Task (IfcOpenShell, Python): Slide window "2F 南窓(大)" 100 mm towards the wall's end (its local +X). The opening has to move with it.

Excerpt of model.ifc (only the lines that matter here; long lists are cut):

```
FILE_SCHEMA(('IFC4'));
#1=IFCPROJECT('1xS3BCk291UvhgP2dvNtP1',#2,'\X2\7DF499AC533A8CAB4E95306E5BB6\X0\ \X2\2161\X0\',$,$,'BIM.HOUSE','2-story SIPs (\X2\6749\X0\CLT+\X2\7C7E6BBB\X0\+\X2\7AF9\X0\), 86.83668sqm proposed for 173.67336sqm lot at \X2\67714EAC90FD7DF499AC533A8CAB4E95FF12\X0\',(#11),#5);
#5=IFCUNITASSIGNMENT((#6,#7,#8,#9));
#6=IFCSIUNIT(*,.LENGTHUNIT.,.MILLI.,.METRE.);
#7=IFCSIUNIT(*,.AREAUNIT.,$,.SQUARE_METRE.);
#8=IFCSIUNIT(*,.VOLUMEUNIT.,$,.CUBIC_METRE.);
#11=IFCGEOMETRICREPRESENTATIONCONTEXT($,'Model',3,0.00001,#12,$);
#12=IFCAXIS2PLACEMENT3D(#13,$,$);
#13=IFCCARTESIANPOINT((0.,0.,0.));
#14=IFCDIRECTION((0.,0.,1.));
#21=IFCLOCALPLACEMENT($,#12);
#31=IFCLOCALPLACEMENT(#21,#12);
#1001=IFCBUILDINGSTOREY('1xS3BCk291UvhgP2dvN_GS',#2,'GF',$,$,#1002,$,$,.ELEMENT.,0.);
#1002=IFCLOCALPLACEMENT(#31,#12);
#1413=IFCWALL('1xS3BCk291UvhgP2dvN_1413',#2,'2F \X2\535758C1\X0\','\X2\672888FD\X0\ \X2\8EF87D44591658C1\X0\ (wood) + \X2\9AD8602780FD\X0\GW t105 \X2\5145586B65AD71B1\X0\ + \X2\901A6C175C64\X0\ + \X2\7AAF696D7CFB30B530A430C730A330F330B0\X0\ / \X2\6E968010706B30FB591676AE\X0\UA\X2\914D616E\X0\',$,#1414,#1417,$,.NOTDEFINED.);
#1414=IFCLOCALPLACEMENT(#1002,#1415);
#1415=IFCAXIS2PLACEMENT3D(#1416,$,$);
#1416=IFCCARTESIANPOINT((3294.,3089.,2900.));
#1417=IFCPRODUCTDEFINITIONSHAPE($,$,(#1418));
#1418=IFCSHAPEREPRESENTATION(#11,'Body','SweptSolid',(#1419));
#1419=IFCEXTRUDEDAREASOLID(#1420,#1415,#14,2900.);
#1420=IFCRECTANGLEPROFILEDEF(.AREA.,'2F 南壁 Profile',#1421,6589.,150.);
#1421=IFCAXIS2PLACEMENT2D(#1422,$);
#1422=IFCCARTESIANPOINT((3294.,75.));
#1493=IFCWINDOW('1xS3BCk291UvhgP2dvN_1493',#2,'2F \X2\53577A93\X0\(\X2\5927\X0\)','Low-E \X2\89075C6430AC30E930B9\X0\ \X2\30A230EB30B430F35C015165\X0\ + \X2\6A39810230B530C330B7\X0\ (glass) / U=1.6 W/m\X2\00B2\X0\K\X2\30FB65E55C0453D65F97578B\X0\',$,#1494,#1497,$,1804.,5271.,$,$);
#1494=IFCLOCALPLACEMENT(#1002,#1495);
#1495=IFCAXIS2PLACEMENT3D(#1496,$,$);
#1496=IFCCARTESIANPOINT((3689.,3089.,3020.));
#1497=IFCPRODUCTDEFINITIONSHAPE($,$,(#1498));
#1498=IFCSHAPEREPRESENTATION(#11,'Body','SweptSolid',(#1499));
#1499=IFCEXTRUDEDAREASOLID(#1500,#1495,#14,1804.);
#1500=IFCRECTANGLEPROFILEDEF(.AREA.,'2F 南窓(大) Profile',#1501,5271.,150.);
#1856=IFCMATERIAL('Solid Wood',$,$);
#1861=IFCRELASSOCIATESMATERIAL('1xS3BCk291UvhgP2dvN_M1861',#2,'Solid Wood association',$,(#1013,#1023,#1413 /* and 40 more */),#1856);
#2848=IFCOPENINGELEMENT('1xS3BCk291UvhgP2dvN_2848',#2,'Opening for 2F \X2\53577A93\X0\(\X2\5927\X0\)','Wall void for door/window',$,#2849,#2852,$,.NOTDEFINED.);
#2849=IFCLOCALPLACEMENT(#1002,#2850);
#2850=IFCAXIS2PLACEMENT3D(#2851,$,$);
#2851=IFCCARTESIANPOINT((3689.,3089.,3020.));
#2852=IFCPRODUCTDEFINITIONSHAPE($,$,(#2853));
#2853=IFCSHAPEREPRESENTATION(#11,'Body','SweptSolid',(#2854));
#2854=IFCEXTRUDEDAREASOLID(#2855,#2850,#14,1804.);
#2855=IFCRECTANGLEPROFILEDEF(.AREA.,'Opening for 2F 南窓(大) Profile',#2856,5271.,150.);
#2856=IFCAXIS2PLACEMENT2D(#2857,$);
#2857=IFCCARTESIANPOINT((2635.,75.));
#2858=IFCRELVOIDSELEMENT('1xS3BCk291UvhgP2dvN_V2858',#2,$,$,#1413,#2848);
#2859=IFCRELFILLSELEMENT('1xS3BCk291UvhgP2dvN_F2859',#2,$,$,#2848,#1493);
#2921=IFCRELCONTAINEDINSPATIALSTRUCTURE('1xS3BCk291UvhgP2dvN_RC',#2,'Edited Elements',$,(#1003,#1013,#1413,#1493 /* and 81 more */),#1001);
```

```python
import ifcopenshell
import ifcopenshell.api.geometry
import ifcopenshell.util.placement
import ifcopenshell.util.unit

model = ifcopenshell.open("model.ifc")
unit_scale = ifcopenshell.util.unit.calculate_unit_scale(model)

window = model.by_guid("1xS3BCk291UvhgP2dvN_1493")
opening = window.FillsVoids[0].RelatingOpeningElement
wall = opening.VoidsElements[0].RelatingBuildingElement

wall_matrix = ifcopenshell.util.placement.get_local_placement(wall.ObjectPlacement)
shift = wall_matrix[:3, 0] * 0.1 / unit_scale
before = ifcopenshell.util.placement.get_local_placement(window.ObjectPlacement)[:3, 3].copy()

# The window is not placed relative to its opening, so move both.
for product in (opening, window):
    matrix = ifcopenshell.util.placement.get_local_placement(product.ObjectPlacement)
    matrix[:3, 3] += shift
    ifcopenshell.api.geometry.edit_object_placement(model, product=product, matrix=matrix, is_si=False)

after = ifcopenshell.util.placement.get_local_placement(window.ObjectPlacement)[:3, 3]
print("window moved by", (after - before).round(3) + 0.0)

model.write("model_v2.ifc")
```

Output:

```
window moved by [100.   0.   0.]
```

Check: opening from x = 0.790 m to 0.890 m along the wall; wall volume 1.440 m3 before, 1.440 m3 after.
